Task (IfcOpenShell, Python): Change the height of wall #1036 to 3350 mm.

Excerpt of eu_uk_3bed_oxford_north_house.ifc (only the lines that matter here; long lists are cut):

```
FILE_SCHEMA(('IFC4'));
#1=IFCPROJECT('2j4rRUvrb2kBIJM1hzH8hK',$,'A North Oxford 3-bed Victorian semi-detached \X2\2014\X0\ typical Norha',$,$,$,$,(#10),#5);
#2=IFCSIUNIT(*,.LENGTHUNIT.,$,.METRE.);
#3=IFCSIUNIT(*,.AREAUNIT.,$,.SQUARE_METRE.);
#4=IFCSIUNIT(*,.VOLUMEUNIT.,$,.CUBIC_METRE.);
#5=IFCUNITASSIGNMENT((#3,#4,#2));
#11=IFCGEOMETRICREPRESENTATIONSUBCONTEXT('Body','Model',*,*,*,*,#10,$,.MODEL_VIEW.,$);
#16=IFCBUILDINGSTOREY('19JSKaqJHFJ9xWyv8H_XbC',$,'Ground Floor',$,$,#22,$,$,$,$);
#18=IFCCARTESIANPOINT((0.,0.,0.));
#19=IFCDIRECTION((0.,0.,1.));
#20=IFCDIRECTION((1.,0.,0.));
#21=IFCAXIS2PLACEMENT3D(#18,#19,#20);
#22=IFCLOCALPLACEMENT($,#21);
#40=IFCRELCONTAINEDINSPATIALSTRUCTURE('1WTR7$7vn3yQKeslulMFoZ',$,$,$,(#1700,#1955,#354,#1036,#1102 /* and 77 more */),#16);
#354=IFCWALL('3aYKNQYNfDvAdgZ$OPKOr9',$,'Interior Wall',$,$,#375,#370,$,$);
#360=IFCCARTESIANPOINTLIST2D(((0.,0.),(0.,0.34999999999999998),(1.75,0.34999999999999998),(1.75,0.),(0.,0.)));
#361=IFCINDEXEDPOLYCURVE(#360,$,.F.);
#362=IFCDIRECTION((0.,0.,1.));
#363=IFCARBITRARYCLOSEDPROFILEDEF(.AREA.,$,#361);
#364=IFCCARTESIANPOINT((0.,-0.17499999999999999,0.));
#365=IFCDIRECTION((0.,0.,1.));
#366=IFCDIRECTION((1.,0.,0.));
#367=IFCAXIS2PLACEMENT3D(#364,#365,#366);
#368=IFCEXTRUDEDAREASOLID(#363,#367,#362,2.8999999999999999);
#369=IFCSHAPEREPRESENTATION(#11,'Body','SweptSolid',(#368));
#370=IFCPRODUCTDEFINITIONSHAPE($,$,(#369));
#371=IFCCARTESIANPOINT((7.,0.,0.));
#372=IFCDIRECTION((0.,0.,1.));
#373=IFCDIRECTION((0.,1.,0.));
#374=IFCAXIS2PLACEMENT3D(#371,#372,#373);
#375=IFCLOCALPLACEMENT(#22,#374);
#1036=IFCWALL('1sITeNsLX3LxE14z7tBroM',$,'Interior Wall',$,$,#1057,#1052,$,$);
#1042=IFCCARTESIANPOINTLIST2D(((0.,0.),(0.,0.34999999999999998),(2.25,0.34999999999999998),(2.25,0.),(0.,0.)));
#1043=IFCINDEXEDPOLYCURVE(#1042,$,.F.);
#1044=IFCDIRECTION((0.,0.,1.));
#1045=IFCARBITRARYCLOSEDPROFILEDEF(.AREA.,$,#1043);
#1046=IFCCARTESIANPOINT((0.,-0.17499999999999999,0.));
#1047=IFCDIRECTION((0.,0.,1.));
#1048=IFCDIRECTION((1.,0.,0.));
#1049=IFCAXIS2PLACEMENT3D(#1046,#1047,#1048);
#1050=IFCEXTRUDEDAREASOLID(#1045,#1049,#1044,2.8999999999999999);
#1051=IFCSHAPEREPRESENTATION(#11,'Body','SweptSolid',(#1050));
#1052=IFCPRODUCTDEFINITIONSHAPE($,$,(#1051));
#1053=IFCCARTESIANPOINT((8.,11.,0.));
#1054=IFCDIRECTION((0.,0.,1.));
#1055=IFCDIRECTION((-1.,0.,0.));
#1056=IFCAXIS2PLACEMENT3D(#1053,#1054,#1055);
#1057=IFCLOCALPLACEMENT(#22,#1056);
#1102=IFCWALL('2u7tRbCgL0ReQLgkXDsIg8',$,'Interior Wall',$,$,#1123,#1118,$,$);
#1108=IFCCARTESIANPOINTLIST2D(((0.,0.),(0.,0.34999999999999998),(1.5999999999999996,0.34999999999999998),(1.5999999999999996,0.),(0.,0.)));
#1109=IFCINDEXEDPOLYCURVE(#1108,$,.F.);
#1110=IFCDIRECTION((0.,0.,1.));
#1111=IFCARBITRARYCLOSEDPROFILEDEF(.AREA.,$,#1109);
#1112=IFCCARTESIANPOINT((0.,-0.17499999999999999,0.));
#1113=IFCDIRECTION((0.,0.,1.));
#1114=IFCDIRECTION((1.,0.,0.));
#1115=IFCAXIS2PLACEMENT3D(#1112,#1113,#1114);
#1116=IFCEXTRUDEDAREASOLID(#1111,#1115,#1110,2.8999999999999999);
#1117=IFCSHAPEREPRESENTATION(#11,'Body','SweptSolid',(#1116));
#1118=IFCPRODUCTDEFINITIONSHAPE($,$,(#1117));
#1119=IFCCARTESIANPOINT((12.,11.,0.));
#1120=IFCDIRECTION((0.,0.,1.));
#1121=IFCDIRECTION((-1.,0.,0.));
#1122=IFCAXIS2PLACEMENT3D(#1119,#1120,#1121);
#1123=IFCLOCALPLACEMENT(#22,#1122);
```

```python
import ifcopenshell
import ifcopenshell.geom
import ifcopenshell.util.representation
import ifcopenshell.util.shape
import ifcopenshell.util.unit

model = ifcopenshell.open("eu_uk_3bed_oxford_north_house.ifc")
unit_scale = ifcopenshell.util.unit.calculate_unit_scale(model)
settings = ifcopenshell.geom.settings()


def volume(element):
    """Net volume in cubic metres, openings subtracted."""
    shape = ifcopenshell.geom.create_shape(settings, element)
    return ifcopenshell.util.shape.get_volume(shape.geometry)


wall = model.by_id(1036)
before = volume(wall)

body = ifcopenshell.util.representation.get_representation(wall, "Model", "Body")
solid = body.Items[0]
old_height = solid.Depth
solid.Depth = 3.35 / unit_scale
after = volume(wall)

print(f"height {old_height:g} -> {solid.Depth:g}, volume {before:.3f} -> {after:.3f} m3")

model.write("eu_uk_3bed_oxford_north_house_v2.ifc")
```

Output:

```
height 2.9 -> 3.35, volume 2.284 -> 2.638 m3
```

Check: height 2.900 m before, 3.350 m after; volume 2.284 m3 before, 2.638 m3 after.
